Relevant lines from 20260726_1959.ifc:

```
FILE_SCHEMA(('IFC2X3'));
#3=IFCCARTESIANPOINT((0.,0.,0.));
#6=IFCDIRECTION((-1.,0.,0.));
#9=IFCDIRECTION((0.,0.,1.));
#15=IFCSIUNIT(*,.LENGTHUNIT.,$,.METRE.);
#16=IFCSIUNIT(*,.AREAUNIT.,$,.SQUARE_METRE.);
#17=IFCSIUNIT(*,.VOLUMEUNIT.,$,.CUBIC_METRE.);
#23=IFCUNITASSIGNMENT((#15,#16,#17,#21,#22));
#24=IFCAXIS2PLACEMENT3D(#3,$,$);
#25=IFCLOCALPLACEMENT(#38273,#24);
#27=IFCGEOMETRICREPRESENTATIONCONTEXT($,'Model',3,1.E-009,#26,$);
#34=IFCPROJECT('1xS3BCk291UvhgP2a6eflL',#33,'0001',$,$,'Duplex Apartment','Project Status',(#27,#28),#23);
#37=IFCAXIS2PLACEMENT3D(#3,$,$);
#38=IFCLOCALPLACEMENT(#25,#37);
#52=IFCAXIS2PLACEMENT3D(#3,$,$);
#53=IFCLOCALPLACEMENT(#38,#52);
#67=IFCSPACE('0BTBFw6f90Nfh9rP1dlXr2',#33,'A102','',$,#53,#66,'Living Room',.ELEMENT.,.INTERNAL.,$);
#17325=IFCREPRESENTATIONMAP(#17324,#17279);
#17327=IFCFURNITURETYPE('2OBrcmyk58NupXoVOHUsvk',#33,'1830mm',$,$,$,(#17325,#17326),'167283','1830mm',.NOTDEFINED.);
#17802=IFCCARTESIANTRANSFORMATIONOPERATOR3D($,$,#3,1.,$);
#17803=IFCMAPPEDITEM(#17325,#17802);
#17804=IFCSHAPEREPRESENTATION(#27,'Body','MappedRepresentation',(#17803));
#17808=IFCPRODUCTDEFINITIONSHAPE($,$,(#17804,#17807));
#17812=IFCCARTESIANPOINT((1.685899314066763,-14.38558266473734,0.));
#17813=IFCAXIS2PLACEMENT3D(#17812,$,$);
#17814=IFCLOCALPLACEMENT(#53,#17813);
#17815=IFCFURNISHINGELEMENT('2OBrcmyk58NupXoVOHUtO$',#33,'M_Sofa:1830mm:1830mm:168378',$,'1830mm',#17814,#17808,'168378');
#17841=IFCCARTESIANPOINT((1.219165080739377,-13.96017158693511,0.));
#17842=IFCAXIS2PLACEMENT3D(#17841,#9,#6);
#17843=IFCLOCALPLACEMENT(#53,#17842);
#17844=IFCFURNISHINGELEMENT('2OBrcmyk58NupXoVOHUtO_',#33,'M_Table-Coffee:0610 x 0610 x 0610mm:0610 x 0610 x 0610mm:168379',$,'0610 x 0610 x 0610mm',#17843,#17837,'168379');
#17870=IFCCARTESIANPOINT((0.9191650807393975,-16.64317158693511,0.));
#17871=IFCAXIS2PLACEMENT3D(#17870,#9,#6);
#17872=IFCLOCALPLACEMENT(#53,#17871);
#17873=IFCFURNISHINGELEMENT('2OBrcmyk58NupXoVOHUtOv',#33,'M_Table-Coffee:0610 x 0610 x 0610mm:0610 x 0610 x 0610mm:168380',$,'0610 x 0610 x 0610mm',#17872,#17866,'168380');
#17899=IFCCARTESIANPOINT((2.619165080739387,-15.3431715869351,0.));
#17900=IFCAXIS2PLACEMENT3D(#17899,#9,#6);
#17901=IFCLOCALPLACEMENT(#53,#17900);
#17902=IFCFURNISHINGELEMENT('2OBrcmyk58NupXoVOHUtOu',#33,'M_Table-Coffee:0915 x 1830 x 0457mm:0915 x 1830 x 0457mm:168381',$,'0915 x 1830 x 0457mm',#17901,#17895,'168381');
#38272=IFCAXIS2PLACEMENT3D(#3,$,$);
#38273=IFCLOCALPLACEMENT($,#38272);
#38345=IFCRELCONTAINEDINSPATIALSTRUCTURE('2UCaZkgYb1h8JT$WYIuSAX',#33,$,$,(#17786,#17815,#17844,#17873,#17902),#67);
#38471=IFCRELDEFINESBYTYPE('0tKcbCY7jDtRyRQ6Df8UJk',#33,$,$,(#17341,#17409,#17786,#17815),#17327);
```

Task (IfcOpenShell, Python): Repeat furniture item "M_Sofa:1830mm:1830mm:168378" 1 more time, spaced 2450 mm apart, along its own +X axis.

```python
import ifcopenshell
import ifcopenshell.api.geometry
import ifcopenshell.api.root
import ifcopenshell.util.element
import ifcopenshell.util.placement

model = ifcopenshell.open("20260726_1959.ifc")


def reuse_history(source, copy):
    """copy_class also copies each property set's owner history, people and application; keep the originals."""
    for rel in copy.IsDefinedBy:
        if rel.is_a("IfcRelDefinesByProperties") and (history := rel.RelatingPropertyDefinition.OwnerHistory):
            rel.RelatingPropertyDefinition.OwnerHistory = source.OwnerHistory
            ifcopenshell.util.element.remove_deep2(model, history)


source = model.by_guid("2OBrcmyk58NupXoVOHUtO$")
base = ifcopenshell.util.placement.get_local_placement(source.ObjectPlacement)
step = base[:3, 0] * 2.45

for i in range(1, 2):
    copy = ifcopenshell.api.root.copy_class(model, product=source)
    copy.Representation = ifcopenshell.util.element.copy_deep(
        model, source.Representation, exclude=["IfcGeometricRepresentationContext", "IfcRepresentationMap"]
    )
    copy.Name = "M_Sofa:1830mm:1830mm"
    copy.Tag = None
    reuse_history(source, copy)
    matrix = base.copy()
    matrix[:3, 3] += i * step
    print("added at", matrix[:3, 3].round(3) + 0.0)
    ifcopenshell.api.geometry.edit_object_placement(model, product=copy, matrix=matrix, is_si=False)

model.write("20260726_1959_rev.ifc")
```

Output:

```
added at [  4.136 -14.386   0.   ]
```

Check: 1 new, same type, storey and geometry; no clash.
